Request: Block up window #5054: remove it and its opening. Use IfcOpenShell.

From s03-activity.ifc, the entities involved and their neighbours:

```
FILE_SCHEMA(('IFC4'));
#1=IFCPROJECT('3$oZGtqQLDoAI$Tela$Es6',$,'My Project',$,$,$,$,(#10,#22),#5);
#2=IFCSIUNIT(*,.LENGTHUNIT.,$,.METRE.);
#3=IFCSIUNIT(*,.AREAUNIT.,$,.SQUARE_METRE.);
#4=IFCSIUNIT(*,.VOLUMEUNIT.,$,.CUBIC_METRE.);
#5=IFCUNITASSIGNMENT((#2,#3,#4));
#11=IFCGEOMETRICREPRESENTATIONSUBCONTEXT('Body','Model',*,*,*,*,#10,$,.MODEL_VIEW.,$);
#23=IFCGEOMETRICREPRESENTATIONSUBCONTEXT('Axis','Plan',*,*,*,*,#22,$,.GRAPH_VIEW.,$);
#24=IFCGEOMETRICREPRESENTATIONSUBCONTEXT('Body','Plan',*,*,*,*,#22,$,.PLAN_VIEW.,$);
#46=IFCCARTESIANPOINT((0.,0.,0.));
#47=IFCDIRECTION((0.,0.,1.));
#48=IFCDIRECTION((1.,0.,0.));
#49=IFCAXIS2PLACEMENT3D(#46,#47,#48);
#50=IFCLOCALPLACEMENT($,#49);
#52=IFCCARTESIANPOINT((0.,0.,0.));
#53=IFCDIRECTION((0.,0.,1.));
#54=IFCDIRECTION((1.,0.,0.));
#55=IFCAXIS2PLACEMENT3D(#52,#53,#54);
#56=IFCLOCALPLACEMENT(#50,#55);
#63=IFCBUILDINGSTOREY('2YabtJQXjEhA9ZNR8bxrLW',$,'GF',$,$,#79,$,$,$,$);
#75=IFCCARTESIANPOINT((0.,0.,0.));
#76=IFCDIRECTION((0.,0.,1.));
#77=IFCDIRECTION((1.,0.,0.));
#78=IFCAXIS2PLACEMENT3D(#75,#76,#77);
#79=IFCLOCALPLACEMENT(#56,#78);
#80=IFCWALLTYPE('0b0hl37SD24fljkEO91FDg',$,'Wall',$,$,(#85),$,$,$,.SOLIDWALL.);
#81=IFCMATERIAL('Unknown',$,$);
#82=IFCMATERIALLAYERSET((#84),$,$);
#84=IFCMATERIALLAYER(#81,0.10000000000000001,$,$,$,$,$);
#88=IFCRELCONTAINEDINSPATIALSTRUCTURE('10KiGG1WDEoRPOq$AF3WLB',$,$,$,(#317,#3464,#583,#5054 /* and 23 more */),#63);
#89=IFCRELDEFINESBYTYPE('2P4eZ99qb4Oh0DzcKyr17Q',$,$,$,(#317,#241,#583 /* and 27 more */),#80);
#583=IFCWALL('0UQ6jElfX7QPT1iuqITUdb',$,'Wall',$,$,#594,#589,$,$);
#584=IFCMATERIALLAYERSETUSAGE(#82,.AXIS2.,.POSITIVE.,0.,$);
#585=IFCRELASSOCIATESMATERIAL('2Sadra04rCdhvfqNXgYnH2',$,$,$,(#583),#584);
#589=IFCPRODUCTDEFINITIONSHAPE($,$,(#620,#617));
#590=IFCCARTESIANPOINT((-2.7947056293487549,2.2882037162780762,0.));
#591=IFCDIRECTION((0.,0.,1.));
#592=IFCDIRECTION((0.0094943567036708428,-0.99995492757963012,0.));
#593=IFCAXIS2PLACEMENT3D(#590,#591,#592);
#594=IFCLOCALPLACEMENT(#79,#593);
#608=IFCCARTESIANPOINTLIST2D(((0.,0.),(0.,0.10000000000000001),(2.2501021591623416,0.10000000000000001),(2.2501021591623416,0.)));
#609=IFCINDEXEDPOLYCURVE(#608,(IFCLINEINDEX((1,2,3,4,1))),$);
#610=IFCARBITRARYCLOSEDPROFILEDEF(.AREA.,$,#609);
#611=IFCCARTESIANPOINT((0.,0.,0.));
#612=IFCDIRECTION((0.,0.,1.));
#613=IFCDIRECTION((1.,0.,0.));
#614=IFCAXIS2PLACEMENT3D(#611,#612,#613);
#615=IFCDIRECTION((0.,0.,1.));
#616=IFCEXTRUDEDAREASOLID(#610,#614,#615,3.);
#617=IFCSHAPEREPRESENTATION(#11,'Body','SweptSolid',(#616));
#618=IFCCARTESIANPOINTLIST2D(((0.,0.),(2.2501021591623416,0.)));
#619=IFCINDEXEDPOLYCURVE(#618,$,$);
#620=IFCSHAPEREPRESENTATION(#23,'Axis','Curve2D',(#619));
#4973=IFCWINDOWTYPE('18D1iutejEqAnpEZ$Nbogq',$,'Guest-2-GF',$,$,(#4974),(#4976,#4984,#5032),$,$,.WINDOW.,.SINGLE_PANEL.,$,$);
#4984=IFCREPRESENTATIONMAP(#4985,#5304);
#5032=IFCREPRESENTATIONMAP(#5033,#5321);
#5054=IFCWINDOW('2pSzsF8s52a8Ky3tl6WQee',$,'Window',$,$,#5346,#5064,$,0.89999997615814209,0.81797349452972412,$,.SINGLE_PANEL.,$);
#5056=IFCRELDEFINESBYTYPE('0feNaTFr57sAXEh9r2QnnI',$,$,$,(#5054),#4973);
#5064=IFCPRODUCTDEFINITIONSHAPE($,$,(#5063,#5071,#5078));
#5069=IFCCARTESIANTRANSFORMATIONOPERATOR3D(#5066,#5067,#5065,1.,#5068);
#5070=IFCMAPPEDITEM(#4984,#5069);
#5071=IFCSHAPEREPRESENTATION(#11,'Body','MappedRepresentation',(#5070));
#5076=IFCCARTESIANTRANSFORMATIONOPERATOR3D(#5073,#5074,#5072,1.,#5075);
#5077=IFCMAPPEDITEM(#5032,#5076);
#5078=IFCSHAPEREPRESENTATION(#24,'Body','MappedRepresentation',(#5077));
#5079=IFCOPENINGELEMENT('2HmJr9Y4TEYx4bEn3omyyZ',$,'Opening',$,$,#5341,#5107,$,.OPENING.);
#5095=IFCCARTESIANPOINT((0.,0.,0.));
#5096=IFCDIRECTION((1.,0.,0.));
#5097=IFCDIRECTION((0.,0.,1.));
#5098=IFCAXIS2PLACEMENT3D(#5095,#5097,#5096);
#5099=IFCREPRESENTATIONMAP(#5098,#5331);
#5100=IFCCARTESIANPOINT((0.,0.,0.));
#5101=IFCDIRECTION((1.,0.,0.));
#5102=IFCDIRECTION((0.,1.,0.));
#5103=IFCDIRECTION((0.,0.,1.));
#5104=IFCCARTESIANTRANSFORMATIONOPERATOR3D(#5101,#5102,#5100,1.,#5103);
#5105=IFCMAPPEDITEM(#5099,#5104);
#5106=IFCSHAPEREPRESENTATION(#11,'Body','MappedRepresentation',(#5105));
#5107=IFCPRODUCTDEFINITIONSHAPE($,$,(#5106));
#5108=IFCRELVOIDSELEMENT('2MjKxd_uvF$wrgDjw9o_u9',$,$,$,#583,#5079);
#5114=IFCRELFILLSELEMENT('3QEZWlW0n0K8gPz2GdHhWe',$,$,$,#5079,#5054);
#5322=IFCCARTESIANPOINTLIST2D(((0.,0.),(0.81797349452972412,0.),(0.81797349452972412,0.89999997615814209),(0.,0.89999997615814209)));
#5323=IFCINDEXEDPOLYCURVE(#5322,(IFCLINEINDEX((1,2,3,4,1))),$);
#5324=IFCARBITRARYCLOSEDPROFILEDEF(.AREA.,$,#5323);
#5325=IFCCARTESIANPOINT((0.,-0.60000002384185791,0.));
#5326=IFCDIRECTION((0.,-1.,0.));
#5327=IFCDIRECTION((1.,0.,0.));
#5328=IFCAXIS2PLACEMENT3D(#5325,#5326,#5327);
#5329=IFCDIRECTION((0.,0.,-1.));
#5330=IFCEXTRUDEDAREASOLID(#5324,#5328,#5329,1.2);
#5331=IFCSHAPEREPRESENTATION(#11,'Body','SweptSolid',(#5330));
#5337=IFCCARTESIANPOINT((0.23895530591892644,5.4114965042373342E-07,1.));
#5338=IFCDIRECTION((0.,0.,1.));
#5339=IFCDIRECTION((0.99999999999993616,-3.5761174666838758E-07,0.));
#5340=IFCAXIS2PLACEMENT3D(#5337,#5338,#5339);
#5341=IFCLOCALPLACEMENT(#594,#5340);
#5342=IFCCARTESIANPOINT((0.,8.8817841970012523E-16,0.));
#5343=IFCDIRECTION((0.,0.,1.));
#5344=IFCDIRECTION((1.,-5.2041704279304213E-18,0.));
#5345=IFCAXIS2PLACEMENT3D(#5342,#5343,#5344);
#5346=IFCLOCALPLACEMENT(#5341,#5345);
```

```python
import ifcopenshell
import ifcopenshell.api.feature
import ifcopenshell.api.root
import ifcopenshell.geom
import ifcopenshell.util.shape

model = ifcopenshell.open("s03-activity.ifc")
settings = ifcopenshell.geom.settings()


def volume(element):
    """Net volume in cubic metres, openings subtracted."""
    shape = ifcopenshell.geom.create_shape(settings, element)
    return ifcopenshell.util.shape.get_volume(shape.geometry)


window = model.by_id(5054)
opening = window.FillsVoids[0].RelatingOpeningElement
wall = opening.VoidsElements[0].RelatingBuildingElement
before = volume(wall)

ifcopenshell.api.root.remove_product(model, product=window)
ifcopenshell.api.feature.remove_feature(model, feature=opening)

after = volume(wall)

print(f"wall volume {before:.3f} -> {after:.3f} m3")

model.write("s03-activity_updated.ifc")
```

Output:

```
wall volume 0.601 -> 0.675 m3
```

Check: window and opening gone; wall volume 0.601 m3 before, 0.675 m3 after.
